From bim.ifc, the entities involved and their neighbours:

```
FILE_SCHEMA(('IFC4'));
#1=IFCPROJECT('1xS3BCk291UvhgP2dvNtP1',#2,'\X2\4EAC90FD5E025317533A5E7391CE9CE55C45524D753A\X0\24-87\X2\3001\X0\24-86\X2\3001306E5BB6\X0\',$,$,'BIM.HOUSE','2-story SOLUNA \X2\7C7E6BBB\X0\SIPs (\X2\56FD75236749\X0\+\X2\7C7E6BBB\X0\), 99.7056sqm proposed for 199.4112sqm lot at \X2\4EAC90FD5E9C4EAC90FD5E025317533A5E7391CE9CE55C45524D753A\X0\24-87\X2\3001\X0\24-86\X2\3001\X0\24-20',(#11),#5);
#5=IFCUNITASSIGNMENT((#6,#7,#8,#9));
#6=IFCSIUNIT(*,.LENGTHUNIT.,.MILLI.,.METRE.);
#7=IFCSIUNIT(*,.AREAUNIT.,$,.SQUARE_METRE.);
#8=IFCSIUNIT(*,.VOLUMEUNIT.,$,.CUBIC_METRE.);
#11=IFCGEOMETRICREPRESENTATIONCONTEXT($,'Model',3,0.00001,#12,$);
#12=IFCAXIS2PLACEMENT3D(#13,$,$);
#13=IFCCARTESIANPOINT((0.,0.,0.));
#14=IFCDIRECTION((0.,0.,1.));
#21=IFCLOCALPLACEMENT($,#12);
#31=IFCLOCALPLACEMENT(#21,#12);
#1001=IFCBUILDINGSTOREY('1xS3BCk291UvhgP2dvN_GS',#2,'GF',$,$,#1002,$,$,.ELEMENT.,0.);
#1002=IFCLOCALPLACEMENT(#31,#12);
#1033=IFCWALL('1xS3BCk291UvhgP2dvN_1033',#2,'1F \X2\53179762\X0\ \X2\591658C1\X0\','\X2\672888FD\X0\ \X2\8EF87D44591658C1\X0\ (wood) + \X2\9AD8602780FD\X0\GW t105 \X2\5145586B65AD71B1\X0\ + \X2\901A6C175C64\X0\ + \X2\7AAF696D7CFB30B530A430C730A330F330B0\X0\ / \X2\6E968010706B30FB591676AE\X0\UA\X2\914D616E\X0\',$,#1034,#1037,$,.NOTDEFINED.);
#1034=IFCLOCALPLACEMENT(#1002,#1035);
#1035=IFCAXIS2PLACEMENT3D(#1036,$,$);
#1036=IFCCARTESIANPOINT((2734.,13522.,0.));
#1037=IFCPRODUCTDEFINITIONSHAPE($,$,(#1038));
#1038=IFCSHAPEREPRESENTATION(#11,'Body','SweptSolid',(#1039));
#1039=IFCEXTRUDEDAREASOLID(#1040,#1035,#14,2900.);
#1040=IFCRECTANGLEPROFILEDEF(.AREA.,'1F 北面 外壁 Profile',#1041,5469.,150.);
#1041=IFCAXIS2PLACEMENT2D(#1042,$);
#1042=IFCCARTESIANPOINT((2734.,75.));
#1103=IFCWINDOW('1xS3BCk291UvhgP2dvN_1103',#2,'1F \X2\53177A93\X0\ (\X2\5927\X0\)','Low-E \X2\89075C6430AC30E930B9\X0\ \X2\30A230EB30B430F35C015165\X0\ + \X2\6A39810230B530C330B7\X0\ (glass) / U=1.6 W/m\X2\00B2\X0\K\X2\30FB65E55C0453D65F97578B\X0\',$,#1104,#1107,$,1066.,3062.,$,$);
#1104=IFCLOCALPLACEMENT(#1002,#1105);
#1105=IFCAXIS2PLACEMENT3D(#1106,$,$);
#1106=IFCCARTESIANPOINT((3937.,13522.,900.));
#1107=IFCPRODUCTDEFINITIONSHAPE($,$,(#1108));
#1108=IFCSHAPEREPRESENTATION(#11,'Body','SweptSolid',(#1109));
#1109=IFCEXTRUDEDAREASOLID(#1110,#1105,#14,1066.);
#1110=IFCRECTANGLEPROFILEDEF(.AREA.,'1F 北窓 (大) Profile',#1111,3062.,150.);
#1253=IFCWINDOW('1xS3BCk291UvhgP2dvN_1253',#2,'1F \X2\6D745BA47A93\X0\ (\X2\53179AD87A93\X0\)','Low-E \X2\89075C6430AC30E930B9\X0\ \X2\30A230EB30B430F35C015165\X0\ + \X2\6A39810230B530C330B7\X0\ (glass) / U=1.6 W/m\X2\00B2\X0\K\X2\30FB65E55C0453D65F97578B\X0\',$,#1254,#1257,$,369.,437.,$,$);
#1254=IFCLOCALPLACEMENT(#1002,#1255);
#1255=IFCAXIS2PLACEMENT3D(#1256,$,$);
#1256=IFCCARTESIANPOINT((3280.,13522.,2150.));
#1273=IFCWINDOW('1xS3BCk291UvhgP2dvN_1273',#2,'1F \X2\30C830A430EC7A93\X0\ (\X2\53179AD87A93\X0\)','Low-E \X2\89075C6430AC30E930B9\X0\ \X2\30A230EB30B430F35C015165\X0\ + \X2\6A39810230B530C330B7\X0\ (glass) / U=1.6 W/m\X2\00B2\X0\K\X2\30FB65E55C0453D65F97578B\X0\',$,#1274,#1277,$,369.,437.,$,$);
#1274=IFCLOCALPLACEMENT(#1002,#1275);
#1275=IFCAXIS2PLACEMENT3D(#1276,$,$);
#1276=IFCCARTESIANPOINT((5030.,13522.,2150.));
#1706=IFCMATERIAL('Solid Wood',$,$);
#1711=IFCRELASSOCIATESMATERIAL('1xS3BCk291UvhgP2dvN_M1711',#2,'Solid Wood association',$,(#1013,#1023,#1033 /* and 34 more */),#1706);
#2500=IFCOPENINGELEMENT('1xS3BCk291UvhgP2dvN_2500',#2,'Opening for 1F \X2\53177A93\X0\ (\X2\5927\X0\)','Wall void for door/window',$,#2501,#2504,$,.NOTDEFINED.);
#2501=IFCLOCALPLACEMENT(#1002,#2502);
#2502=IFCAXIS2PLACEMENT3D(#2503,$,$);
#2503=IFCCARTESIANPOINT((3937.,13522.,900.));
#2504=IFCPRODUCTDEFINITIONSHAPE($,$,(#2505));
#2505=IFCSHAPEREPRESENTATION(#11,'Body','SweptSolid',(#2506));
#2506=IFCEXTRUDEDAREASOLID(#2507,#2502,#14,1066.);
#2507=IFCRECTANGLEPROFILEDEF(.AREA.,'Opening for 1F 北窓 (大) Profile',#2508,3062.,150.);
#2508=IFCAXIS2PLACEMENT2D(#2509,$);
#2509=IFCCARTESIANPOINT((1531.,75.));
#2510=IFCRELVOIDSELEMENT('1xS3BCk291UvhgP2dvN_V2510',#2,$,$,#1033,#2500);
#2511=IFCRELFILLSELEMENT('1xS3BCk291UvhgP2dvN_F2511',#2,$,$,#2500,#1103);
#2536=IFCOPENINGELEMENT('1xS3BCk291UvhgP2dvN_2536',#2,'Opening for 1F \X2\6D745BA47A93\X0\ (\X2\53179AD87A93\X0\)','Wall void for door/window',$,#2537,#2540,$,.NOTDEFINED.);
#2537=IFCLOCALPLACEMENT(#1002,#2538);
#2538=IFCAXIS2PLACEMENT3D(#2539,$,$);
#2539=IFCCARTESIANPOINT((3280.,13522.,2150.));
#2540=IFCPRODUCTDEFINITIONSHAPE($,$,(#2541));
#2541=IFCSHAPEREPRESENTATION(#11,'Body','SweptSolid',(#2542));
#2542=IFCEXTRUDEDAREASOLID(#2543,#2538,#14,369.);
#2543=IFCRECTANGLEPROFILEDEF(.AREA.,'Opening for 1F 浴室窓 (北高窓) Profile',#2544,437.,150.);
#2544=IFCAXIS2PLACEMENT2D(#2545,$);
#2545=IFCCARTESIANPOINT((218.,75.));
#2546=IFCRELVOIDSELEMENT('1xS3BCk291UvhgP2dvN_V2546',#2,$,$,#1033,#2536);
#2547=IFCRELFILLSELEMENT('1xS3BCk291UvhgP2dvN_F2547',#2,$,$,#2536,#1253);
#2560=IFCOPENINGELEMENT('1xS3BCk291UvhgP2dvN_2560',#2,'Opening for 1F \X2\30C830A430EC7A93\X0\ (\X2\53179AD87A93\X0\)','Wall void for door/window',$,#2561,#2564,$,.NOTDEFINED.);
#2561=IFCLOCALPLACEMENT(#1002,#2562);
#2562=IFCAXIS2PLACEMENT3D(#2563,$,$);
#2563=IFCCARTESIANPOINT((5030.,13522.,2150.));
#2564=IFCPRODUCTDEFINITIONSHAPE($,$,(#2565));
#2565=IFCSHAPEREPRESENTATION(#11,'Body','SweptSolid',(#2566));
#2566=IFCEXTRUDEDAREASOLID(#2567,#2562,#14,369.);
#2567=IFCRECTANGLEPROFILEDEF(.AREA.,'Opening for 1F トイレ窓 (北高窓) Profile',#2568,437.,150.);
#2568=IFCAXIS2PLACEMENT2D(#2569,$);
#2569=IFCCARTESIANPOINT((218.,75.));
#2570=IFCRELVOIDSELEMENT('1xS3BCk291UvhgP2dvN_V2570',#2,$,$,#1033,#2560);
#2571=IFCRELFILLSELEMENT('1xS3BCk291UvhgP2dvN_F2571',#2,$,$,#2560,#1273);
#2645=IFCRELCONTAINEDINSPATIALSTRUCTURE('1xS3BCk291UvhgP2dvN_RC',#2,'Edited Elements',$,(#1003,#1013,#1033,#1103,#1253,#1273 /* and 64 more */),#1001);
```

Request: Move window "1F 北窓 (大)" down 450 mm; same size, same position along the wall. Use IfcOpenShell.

```python
import numpy as np
import ifcopenshell
import ifcopenshell.api.geometry
import ifcopenshell.util.placement
import ifcopenshell.util.unit

model = ifcopenshell.open("bim.ifc")
unit_scale = ifcopenshell.util.unit.calculate_unit_scale(model)

window = model.by_id(1103)
opening = window.FillsVoids[0].RelatingOpeningElement
dz = -0.45 / unit_scale

shift = np.array([0.0, 0.0, dz])
# The window is not placed relative to its opening, so move both.
for product in (opening, window):
    matrix = ifcopenshell.util.placement.get_local_placement(product.ObjectPlacement)
    matrix[:3, 3] += shift
    ifcopenshell.api.geometry.edit_object_placement(model, product=product, matrix=matrix, is_si=False)

print(f"moved by {dz * unit_scale:+.3f} m")

model.write("bim_rev.ifc")
```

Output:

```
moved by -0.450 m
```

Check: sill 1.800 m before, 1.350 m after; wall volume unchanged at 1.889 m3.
